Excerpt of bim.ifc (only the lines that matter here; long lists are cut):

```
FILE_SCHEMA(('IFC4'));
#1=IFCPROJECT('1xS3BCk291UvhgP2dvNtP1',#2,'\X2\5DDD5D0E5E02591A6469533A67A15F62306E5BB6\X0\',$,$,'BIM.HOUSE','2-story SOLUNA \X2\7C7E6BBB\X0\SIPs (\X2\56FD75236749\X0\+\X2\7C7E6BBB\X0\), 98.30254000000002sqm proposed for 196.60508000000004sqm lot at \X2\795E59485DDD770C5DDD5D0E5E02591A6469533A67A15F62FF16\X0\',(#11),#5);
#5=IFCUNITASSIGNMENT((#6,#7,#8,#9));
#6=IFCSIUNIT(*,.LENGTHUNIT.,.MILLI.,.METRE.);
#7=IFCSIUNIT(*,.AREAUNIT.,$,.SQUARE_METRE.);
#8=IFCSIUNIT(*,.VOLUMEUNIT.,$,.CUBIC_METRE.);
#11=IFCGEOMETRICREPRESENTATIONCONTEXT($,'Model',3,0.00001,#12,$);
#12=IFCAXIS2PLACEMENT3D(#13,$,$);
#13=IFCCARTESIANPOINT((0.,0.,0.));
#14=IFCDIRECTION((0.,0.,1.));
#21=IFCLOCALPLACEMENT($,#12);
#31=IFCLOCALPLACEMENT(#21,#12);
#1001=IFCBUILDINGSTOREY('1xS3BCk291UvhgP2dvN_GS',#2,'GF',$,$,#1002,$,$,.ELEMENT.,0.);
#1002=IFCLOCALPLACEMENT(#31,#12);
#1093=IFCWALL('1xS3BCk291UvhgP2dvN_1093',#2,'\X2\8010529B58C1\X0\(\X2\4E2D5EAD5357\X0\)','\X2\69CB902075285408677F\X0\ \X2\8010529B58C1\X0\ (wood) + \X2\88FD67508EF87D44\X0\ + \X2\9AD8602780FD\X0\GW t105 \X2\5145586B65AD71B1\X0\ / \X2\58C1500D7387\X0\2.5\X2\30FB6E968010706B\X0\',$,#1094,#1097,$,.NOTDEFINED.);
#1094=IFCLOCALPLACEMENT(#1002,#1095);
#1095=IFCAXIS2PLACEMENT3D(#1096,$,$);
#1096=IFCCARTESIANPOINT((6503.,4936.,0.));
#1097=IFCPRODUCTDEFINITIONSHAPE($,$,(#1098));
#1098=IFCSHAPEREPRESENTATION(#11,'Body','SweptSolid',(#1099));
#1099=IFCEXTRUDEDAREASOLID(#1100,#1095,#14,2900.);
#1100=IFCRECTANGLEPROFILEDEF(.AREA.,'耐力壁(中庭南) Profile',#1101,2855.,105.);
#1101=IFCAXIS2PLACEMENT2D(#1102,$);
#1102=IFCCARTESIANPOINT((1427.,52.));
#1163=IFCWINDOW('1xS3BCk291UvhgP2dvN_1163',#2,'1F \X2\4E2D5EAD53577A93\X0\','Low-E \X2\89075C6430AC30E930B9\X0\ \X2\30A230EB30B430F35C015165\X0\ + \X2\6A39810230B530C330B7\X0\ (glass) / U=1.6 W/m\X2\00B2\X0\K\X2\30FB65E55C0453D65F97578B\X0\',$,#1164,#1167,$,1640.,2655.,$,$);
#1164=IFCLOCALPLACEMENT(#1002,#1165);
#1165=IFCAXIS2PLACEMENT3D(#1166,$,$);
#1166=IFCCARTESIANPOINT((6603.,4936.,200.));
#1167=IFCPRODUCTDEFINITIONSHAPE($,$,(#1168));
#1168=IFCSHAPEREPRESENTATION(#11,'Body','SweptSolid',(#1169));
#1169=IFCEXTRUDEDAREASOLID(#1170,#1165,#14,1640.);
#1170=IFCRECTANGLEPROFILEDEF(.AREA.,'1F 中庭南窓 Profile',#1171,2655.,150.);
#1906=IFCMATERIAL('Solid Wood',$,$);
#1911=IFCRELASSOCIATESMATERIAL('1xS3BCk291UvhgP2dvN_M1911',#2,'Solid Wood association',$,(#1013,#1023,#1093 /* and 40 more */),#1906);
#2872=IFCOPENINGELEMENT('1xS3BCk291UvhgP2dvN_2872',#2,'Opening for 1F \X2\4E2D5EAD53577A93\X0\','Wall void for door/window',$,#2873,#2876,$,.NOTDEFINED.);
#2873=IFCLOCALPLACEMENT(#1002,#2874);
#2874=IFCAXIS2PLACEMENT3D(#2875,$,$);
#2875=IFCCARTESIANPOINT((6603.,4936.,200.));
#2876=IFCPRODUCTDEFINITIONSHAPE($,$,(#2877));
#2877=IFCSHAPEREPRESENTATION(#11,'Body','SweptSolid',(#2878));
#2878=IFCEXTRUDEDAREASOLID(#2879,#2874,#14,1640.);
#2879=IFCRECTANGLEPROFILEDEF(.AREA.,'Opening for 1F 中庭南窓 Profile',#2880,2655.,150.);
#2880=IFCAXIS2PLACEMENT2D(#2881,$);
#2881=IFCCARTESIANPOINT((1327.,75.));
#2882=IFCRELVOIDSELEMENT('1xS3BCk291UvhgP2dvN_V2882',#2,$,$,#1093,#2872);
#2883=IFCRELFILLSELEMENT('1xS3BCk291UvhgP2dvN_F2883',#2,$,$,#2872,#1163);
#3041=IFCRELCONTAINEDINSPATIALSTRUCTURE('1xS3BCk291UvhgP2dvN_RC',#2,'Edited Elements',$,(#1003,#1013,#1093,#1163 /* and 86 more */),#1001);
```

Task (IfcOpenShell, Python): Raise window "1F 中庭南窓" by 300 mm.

```python
import numpy as np
import ifcopenshell
import ifcopenshell.api.geometry
import ifcopenshell.util.placement
import ifcopenshell.util.unit

model = ifcopenshell.open("bim.ifc")
unit_scale = ifcopenshell.util.unit.calculate_unit_scale(model)

window = model.by_guid("1xS3BCk291UvhgP2dvN_1163")
opening = window.FillsVoids[0].RelatingOpeningElement
dz = 300.0

shift = np.array([0.0, 0.0, dz])
# The window is not placed relative to its opening, so move both.
for product in (opening, window):
    matrix = ifcopenshell.util.placement.get_local_placement(product.ObjectPlacement)
    matrix[:3, 3] += shift
    ifcopenshell.api.geometry.edit_object_placement(model, product=product, matrix=matrix, is_si=False)

print(f"moved by {dz * unit_scale:+.3f} m")

model.write("bim_updated.ifc")
```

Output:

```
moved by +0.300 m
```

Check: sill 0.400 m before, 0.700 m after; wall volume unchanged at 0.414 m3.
